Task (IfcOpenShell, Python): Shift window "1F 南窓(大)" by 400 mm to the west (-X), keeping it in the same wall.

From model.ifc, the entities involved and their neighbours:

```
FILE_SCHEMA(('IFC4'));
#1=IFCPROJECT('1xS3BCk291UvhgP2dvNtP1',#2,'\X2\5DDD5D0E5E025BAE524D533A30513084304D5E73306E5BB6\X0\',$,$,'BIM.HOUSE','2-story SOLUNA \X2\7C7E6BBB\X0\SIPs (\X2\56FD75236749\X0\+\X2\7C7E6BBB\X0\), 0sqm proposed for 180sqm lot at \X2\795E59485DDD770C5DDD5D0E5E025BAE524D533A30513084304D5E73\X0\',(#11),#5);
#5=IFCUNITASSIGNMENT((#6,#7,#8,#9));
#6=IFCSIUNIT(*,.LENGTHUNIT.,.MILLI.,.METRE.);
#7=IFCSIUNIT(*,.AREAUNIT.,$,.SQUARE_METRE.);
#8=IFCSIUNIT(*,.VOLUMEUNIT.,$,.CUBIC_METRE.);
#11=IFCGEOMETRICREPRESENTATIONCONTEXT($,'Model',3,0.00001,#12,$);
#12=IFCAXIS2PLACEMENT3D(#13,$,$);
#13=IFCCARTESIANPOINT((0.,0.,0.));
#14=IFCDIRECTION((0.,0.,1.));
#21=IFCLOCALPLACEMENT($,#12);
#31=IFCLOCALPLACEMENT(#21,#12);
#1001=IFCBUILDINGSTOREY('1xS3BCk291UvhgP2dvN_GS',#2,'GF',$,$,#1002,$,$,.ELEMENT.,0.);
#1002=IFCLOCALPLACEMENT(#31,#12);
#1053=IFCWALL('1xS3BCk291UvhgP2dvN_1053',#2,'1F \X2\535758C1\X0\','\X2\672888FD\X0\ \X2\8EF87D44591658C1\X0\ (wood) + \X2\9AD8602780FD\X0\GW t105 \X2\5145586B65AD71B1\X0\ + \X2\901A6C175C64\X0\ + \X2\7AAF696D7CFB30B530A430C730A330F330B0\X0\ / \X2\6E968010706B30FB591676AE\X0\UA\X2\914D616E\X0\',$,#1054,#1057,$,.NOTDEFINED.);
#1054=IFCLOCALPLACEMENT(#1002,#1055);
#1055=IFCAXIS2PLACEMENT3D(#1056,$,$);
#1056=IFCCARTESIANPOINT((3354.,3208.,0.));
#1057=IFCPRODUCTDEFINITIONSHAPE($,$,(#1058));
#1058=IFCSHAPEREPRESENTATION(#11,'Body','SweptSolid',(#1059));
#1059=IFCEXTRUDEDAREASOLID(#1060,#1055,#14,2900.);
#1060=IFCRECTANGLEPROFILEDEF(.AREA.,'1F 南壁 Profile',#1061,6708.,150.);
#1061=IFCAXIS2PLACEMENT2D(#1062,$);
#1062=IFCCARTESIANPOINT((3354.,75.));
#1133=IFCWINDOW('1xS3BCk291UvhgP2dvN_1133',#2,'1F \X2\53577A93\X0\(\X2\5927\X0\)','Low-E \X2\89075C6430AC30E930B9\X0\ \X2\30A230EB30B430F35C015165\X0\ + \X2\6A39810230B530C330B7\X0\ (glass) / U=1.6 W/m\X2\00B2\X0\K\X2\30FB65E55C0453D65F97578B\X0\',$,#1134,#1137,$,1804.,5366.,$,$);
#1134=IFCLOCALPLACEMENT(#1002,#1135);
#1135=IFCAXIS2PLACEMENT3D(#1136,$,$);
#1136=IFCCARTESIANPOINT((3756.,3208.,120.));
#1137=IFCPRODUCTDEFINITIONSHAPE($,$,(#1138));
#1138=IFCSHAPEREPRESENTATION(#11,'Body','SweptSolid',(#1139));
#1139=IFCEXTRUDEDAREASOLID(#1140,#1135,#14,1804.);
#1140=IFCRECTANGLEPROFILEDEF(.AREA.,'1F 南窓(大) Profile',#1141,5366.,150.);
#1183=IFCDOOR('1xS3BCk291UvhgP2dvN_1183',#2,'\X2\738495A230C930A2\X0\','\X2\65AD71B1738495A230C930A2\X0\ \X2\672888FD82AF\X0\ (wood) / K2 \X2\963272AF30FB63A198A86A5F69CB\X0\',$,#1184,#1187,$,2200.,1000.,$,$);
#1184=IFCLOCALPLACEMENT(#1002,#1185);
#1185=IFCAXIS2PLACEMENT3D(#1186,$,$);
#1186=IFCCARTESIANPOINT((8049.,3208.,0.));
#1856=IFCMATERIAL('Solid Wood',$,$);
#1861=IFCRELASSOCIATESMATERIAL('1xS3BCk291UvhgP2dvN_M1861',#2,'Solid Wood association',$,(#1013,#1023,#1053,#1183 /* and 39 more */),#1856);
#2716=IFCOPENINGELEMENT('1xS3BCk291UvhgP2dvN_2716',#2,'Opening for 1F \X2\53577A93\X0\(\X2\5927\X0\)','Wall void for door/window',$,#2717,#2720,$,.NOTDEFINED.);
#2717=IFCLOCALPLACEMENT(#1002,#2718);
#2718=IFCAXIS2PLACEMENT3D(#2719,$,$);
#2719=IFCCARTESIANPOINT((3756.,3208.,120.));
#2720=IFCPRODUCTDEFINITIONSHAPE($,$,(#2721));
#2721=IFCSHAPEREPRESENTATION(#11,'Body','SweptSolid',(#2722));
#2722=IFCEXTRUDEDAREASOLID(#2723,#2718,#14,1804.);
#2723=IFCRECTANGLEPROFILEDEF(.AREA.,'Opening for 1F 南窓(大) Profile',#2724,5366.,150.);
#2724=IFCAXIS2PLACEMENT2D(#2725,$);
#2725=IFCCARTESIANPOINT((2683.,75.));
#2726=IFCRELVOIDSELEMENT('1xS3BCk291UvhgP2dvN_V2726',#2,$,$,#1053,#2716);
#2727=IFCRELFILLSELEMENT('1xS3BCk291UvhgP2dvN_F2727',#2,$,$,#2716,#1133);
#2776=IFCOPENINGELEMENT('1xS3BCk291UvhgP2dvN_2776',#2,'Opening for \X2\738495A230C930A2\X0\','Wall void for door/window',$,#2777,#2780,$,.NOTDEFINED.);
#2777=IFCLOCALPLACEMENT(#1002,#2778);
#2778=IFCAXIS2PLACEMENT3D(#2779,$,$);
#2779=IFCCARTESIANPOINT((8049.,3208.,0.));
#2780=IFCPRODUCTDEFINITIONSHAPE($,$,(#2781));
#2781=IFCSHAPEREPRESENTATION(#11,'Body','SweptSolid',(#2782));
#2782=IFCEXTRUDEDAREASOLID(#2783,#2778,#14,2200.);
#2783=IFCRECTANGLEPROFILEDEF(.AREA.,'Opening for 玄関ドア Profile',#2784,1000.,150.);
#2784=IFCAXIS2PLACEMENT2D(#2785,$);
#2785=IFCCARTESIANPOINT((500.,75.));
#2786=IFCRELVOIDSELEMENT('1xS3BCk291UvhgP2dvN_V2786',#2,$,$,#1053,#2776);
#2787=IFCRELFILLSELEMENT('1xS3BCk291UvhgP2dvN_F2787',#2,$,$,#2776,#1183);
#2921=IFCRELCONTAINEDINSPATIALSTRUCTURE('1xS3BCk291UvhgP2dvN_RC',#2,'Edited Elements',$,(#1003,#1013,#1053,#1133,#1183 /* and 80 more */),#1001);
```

```python
import ifcopenshell
import ifcopenshell.api.geometry
import ifcopenshell.util.placement

model = ifcopenshell.open("model.ifc")

window = model.by_id(1133)
opening = window.FillsVoids[0].RelatingOpeningElement
wall = opening.VoidsElements[0].RelatingBuildingElement

wall_matrix = ifcopenshell.util.placement.get_local_placement(wall.ObjectPlacement)
shift = wall_matrix[:3, 0] * -400.0
before = ifcopenshell.util.placement.get_local_placement(window.ObjectPlacement)[:3, 3].copy()

# The window is not placed relative to its opening, so move both.
for product in (opening, window):
    matrix = ifcopenshell.util.placement.get_local_placement(product.ObjectPlacement)
    matrix[:3, 3] += shift
    ifcopenshell.api.geometry.edit_object_placement(model, product=product, matrix=matrix, is_si=False)

after = ifcopenshell.util.placement.get_local_placement(window.ObjectPlacement)[:3, 3]
print("window moved by", (after - before).round(3) + 0.0)

model.write("model-out.ifc")
```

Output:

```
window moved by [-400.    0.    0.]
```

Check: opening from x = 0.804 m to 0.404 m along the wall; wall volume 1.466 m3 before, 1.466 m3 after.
